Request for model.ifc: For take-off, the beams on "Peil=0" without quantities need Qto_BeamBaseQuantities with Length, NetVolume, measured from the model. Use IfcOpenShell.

First a look at what the model holds.

```python
import ifcopenshell
import ifcopenshell.util.element
import ifcopenshell.util.unit

model = ifcopenshell.open("model.ifc")
print(model.schema)
for unit_type in ("LENGTHUNIT", "AREAUNIT", "VOLUMEUNIT"):
    print(unit_type, ifcopenshell.util.unit.calculate_unit_scale(model, unit_type))
storey = next(s for s in model.by_type("IfcBuildingStorey") if s.Name == "Peil=0")
beams = [e for e in ifcopenshell.util.element.get_decomposition(storey) if e.is_a("IfcBeam")]
for e in sorted(beams, key=lambda e: e.id()):
    print(e.id(), e.is_a(), e.Name, list(ifcopenshell.util.element.get_psets(e, qtos_only=True)), sep=" | ")
```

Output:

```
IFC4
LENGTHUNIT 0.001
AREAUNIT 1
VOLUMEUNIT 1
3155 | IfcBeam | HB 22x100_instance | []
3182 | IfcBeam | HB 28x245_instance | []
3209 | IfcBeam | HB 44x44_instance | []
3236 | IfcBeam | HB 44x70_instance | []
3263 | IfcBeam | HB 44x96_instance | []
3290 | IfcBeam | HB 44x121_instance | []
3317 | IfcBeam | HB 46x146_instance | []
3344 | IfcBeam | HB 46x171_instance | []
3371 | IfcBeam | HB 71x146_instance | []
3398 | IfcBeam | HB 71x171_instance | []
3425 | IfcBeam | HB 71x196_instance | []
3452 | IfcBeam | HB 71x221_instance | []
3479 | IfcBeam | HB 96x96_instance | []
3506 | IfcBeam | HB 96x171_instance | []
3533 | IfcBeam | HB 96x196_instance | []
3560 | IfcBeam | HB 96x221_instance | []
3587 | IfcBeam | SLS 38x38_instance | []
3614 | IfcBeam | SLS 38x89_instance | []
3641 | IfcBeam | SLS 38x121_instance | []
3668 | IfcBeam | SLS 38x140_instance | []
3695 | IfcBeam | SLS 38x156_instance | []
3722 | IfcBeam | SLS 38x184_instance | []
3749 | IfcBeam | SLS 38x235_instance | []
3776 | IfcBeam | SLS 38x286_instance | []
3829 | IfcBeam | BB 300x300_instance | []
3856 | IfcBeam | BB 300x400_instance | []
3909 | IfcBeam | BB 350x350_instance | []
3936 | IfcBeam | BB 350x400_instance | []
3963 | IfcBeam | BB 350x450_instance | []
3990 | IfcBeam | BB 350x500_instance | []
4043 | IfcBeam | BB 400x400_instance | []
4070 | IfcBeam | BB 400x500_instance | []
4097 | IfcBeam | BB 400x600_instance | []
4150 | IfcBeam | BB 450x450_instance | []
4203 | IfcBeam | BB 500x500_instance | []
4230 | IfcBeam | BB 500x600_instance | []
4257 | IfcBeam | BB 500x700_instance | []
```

```python
import ifcopenshell
import ifcopenshell.api.pset
import ifcopenshell.geom
import ifcopenshell.util.element
import ifcopenshell.util.shape
import ifcopenshell.util.unit

model = ifcopenshell.open("model.ifc")
unit_scale = ifcopenshell.util.unit.calculate_unit_scale(model)
volume_scale = ifcopenshell.util.unit.calculate_unit_scale(model, "VOLUMEUNIT")
settings = ifcopenshell.geom.settings()

storey = next(s for s in model.by_type("IfcBuildingStorey") if s.Name == "Peil=0")
beams = [e for e in ifcopenshell.util.element.get_decomposition(storey) if e.is_a("IfcBeam")]

for e in sorted(beams, key=lambda e: e.id()):
    if ifcopenshell.util.element.get_psets(e, qtos_only=True, should_inherit=False):
        continue
    # Geometry comes back in metres, in the element's own axes.
    shape = ifcopenshell.geom.create_shape(settings, e)
    values = {
        "Length": ifcopenshell.util.shape.get_max_xyz(shape.geometry) / unit_scale,
        "NetVolume": ifcopenshell.util.shape.get_volume(shape.geometry) / volume_scale,
    }
    qto = ifcopenshell.api.pset.add_qto(model, product=e, name="Qto_BeamBaseQuantities")
    ifcopenshell.api.pset.edit_qto(model, qto=qto, properties=values)
    print(e.id(), {k: round(v, 3) for k, v in values.items()})

model.write("model_edited.ifc")
```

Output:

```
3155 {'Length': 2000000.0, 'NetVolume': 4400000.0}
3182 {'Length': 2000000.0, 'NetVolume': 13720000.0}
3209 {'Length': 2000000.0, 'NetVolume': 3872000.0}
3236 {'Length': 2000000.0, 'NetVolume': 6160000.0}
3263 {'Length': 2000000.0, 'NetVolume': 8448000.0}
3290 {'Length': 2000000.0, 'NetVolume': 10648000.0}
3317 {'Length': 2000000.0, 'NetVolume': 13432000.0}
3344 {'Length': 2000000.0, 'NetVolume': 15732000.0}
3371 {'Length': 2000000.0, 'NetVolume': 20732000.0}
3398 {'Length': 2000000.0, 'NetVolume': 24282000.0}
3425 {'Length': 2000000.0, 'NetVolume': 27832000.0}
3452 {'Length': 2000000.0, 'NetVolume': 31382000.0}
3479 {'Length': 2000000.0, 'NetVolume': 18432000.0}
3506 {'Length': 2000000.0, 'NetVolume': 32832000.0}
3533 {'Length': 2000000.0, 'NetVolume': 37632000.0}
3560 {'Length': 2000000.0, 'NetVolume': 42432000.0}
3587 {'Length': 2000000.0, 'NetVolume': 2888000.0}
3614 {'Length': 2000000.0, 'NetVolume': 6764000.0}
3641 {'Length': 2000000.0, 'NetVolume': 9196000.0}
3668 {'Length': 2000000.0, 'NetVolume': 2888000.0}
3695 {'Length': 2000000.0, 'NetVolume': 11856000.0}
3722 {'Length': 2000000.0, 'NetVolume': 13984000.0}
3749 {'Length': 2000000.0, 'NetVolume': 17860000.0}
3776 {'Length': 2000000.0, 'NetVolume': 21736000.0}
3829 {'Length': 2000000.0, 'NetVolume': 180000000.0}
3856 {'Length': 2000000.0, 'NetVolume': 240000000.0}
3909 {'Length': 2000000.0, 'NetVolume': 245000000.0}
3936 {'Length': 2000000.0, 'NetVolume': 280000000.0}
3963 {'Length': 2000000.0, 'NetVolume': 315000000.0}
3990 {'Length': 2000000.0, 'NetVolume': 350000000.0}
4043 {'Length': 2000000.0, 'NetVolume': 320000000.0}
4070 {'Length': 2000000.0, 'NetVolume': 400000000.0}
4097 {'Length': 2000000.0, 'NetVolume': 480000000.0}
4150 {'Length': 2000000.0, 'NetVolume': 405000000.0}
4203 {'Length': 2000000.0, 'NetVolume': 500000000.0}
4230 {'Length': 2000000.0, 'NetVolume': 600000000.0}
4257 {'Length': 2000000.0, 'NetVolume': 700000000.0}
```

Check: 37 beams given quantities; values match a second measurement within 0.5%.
